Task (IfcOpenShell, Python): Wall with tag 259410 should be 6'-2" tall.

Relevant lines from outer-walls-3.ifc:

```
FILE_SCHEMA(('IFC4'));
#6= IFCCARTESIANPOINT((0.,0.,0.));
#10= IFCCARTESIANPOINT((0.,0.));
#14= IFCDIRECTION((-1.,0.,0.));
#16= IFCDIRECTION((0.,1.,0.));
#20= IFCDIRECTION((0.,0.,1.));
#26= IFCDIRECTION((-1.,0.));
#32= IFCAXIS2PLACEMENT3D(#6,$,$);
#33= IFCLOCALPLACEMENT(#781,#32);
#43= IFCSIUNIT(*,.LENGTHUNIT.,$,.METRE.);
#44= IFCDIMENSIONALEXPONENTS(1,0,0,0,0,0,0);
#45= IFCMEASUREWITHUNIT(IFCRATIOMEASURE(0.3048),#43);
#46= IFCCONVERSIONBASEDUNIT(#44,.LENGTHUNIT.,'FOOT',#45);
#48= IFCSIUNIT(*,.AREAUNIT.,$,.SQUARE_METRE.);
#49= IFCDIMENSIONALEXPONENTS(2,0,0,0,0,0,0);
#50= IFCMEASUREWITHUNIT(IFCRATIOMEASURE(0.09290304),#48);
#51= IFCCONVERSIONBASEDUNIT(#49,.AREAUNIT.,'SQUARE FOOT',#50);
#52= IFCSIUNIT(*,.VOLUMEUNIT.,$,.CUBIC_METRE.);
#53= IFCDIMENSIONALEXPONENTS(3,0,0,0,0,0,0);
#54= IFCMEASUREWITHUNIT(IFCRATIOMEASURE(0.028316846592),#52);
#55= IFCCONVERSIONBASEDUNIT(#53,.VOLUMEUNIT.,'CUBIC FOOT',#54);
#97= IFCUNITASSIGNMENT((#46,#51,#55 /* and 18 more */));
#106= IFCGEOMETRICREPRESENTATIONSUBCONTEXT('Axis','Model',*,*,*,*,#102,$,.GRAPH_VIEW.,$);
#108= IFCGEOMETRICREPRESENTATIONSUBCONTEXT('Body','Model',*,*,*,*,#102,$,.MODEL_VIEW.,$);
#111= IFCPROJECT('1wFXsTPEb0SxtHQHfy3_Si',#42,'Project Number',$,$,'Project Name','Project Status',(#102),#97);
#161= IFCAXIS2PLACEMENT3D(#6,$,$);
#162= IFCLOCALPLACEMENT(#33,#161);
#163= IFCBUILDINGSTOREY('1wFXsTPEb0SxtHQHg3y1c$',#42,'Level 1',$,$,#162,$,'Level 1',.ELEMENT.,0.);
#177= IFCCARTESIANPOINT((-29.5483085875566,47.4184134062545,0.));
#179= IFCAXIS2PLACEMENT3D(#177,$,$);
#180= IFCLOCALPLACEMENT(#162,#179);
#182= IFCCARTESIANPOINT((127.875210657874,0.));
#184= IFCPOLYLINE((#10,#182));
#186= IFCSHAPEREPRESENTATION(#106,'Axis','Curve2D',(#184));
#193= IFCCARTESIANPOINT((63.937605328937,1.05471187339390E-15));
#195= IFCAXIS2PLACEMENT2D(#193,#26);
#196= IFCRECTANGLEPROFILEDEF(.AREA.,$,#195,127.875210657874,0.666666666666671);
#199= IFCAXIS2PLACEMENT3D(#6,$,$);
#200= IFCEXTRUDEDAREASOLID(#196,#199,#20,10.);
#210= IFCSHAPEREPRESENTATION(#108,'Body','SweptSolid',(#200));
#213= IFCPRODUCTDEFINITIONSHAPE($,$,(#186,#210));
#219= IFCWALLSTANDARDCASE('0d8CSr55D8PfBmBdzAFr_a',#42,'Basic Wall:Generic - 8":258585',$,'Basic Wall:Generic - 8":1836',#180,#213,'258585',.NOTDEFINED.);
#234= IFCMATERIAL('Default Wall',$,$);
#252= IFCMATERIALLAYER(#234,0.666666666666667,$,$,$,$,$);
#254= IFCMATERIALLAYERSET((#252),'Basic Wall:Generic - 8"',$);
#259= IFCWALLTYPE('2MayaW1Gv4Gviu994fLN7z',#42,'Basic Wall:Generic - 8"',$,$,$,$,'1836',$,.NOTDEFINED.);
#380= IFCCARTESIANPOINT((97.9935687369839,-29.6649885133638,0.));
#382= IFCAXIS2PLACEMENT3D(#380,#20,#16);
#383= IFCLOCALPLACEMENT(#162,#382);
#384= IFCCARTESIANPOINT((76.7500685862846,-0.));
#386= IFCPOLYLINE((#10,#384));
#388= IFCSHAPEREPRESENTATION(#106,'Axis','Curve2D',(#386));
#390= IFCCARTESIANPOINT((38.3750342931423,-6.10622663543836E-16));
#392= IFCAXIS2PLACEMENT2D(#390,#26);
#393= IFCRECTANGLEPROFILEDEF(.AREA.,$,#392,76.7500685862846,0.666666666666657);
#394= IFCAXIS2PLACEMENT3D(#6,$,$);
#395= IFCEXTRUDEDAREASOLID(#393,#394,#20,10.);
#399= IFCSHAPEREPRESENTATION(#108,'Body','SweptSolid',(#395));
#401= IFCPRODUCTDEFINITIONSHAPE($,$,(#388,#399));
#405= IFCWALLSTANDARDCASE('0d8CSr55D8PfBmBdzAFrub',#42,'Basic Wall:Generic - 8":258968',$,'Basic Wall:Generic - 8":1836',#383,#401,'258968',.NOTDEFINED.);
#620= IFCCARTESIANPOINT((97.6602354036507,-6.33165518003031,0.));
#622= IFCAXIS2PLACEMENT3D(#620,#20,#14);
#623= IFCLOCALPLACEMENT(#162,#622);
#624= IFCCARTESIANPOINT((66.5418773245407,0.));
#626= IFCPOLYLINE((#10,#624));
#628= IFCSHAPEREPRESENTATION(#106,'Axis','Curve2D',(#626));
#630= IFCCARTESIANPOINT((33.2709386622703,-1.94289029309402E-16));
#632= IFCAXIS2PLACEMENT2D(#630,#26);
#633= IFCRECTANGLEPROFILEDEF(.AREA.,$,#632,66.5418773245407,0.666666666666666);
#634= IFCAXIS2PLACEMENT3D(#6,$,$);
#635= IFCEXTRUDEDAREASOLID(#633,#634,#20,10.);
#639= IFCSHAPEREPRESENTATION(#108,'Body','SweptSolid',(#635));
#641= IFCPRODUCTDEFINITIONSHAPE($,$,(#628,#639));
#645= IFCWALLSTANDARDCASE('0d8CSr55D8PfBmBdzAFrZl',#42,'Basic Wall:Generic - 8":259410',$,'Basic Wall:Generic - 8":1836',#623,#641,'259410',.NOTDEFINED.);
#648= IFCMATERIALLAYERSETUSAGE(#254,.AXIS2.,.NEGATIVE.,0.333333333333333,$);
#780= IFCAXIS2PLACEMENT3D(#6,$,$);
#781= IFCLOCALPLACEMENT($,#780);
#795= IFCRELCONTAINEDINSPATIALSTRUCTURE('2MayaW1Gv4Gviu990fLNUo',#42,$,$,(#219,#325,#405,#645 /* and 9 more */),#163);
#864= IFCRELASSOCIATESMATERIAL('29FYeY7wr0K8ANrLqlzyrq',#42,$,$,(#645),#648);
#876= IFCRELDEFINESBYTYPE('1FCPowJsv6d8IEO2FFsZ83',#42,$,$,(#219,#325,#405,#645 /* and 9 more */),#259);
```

```python
import ifcopenshell
import ifcopenshell.geom
import ifcopenshell.util.representation
import ifcopenshell.util.shape
import ifcopenshell.util.unit

model = ifcopenshell.open("outer-walls-3.ifc")
unit_scale = ifcopenshell.util.unit.calculate_unit_scale(model)
settings = ifcopenshell.geom.settings()


def volume(element):
    """Net volume in cubic metres, openings subtracted."""
    shape = ifcopenshell.geom.create_shape(settings, element)
    return ifcopenshell.util.shape.get_volume(shape.geometry)


wall = model.by_guid("0d8CSr55D8PfBmBdzAFrZl")
before = volume(wall)

body = ifcopenshell.util.representation.get_representation(wall, "Model", "Body")
solid = body.Items[0]
old_height = solid.Depth
solid.Depth = 74 * 0.0254 / unit_scale
after = volume(wall)

print(f"height {old_height:g} -> {solid.Depth:g}, volume {before:.3f} -> {after:.3f} m3")

model.write("outer-walls-3-out.ifc")
```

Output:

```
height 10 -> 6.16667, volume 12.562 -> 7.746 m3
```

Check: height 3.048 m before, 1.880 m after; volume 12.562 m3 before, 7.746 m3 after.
